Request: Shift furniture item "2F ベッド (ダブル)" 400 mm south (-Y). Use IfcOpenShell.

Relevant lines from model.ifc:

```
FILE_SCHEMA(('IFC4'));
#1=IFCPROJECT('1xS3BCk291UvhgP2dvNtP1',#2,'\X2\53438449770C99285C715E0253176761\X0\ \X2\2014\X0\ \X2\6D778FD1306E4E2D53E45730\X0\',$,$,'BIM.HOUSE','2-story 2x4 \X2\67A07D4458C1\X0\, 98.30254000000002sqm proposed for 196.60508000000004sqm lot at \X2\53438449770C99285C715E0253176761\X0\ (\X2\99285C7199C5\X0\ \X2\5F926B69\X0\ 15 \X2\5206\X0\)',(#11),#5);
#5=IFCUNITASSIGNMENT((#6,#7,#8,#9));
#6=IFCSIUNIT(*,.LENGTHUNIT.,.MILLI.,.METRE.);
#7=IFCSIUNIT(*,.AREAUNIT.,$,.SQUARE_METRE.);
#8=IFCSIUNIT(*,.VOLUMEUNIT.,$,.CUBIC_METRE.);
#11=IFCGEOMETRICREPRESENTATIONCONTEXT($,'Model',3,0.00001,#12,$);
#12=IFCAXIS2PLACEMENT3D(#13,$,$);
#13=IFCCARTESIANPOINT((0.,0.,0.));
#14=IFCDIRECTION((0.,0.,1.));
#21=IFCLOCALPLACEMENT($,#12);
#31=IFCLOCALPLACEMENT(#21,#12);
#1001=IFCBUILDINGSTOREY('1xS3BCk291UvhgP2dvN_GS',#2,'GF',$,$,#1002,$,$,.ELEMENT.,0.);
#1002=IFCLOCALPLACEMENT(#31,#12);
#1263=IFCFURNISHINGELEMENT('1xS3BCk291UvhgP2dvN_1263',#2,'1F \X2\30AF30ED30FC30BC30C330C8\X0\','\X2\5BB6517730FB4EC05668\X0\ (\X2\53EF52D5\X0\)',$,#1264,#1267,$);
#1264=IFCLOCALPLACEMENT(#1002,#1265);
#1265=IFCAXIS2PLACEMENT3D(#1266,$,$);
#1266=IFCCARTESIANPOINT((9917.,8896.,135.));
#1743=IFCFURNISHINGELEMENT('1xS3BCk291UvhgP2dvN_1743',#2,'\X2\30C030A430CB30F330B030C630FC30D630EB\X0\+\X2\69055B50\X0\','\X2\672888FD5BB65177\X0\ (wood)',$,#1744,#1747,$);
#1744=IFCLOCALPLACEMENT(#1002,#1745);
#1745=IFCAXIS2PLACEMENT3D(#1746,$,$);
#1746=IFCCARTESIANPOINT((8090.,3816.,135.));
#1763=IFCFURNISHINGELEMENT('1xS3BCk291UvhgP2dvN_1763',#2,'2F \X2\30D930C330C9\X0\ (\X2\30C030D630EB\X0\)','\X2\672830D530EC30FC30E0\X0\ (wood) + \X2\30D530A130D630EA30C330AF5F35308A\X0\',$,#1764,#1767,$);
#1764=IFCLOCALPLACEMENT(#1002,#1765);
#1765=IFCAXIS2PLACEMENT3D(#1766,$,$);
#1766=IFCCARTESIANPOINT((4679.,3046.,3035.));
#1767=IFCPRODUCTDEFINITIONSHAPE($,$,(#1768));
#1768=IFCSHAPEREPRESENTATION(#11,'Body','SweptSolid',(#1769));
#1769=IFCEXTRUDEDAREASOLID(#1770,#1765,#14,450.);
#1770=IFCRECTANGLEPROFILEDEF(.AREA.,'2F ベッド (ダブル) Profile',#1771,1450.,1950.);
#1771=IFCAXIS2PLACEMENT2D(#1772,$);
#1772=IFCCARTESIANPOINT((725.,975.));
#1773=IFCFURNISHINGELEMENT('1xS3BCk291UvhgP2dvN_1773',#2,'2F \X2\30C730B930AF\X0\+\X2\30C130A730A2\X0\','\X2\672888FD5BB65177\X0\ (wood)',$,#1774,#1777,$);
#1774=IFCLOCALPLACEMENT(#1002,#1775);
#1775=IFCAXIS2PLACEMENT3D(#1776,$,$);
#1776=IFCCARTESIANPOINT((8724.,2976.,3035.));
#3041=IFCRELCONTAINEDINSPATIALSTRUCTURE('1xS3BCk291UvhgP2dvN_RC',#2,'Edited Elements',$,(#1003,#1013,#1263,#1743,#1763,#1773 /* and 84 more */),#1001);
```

```python
import ifcopenshell
import ifcopenshell.api.geometry
import ifcopenshell.util.placement
import ifcopenshell.util.unit

model = ifcopenshell.open("model.ifc")
unit_scale = ifcopenshell.util.unit.calculate_unit_scale(model)

item = model.by_id(1763)
matrix = ifcopenshell.util.placement.get_local_placement(item.ObjectPlacement)
matrix[1, 3] -= 0.4 / unit_scale
ifcopenshell.api.geometry.edit_object_placement(model, product=item, matrix=matrix, is_si=False)

print(ifcopenshell.util.placement.get_local_placement(item.ObjectPlacement).round(3) + 0.0)

model.write("model_v2.ifc")
```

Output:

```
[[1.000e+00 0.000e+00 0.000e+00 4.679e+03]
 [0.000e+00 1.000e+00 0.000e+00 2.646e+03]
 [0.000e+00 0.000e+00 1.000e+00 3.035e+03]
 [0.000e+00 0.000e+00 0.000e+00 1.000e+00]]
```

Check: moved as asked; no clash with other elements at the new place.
